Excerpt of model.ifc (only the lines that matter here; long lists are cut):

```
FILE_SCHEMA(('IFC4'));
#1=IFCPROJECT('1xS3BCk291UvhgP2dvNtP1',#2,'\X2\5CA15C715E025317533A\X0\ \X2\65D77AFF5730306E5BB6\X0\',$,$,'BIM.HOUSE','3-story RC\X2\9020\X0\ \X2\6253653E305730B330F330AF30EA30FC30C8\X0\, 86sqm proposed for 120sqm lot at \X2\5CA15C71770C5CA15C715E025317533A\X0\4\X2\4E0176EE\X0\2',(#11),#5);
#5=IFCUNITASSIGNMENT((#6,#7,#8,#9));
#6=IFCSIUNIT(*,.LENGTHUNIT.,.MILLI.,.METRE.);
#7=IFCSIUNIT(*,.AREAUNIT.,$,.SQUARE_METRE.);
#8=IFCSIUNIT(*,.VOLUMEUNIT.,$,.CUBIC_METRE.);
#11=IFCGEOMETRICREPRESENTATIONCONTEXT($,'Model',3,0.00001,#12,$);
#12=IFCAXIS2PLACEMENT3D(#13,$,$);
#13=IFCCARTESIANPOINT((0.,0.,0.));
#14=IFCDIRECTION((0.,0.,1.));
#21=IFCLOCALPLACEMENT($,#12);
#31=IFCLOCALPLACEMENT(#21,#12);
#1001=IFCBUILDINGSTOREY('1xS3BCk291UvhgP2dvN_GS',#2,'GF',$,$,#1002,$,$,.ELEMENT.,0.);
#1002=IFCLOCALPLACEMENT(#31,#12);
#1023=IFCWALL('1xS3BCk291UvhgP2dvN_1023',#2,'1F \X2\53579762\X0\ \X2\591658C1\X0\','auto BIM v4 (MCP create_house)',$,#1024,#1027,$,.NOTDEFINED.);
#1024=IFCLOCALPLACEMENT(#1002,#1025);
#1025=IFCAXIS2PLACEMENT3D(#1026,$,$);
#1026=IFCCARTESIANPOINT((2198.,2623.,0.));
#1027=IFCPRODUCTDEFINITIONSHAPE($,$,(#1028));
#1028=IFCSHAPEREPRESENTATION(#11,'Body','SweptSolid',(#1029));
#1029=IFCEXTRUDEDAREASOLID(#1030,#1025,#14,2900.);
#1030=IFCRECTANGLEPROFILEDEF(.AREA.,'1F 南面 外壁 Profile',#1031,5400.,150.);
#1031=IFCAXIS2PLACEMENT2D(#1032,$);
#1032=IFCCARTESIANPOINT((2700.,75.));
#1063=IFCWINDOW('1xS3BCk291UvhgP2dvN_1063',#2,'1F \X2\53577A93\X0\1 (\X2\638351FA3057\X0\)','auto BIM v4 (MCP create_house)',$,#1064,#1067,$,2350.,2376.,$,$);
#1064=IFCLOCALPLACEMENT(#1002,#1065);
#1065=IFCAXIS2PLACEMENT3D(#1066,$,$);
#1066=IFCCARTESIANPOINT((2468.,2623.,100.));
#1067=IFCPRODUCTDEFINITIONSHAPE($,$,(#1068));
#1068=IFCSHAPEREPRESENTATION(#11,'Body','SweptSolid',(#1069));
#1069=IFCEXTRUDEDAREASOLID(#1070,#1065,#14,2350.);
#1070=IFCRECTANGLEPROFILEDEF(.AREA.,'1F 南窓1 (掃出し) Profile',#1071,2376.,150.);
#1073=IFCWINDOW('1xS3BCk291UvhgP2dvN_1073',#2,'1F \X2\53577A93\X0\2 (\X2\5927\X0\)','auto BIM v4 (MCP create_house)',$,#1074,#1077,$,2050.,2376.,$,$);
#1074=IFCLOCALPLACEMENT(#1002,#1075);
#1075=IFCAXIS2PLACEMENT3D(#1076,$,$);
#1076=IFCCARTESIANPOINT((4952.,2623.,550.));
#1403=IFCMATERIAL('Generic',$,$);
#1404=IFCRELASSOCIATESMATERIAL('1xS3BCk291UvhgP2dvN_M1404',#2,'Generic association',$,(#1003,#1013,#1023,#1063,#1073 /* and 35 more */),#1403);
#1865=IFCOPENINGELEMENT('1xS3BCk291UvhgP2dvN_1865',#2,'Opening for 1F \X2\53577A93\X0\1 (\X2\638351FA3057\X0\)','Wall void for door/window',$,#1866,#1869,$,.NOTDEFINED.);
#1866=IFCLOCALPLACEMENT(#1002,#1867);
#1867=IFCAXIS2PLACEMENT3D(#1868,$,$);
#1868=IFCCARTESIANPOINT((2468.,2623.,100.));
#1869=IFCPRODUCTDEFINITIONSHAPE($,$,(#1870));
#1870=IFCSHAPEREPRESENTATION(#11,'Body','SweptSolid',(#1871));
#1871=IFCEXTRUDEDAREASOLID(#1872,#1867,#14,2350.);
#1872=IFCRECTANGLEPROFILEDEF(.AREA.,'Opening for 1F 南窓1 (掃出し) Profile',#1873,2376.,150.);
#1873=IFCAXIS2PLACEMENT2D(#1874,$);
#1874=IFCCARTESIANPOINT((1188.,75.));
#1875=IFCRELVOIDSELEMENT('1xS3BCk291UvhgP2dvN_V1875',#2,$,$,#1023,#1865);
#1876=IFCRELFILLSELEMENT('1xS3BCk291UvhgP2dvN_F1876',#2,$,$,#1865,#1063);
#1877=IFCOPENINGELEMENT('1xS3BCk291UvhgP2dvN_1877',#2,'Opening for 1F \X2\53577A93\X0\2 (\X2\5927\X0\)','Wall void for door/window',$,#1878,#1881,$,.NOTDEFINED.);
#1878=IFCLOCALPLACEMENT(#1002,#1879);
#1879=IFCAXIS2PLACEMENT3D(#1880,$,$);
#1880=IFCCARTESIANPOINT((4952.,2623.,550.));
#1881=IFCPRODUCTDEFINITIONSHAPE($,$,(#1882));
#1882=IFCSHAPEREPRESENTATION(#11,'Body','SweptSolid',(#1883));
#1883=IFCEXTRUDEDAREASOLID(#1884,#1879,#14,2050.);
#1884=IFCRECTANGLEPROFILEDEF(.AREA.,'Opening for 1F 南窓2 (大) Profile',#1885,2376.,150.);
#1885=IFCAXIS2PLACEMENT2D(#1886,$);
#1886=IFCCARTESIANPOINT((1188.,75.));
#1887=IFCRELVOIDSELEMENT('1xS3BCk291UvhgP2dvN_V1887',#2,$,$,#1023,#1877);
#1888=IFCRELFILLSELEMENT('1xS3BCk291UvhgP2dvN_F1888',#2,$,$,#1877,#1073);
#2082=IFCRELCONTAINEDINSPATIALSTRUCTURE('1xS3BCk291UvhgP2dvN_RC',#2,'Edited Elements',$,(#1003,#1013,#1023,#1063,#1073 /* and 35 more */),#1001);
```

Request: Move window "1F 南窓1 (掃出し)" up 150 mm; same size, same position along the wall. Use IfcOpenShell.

```python
import numpy as np
import ifcopenshell
import ifcopenshell.api.geometry
import ifcopenshell.util.placement
import ifcopenshell.util.unit

model = ifcopenshell.open("model.ifc")
unit_scale = ifcopenshell.util.unit.calculate_unit_scale(model)

window = model.by_guid("1xS3BCk291UvhgP2dvN_1063")
opening = window.FillsVoids[0].RelatingOpeningElement
dz = 150.0

shift = np.array([0.0, 0.0, dz])
# The window is not placed relative to its opening, so move both.
for product in (opening, window):
    matrix = ifcopenshell.util.placement.get_local_placement(product.ObjectPlacement)
    matrix[:3, 3] += shift
    ifcopenshell.api.geometry.edit_object_placement(model, product=product, matrix=matrix, is_si=False)

print(f"moved by {dz * unit_scale:+.3f} m")

model.write("model_edited.ifc")
```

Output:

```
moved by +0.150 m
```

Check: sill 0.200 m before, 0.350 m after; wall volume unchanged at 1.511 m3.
